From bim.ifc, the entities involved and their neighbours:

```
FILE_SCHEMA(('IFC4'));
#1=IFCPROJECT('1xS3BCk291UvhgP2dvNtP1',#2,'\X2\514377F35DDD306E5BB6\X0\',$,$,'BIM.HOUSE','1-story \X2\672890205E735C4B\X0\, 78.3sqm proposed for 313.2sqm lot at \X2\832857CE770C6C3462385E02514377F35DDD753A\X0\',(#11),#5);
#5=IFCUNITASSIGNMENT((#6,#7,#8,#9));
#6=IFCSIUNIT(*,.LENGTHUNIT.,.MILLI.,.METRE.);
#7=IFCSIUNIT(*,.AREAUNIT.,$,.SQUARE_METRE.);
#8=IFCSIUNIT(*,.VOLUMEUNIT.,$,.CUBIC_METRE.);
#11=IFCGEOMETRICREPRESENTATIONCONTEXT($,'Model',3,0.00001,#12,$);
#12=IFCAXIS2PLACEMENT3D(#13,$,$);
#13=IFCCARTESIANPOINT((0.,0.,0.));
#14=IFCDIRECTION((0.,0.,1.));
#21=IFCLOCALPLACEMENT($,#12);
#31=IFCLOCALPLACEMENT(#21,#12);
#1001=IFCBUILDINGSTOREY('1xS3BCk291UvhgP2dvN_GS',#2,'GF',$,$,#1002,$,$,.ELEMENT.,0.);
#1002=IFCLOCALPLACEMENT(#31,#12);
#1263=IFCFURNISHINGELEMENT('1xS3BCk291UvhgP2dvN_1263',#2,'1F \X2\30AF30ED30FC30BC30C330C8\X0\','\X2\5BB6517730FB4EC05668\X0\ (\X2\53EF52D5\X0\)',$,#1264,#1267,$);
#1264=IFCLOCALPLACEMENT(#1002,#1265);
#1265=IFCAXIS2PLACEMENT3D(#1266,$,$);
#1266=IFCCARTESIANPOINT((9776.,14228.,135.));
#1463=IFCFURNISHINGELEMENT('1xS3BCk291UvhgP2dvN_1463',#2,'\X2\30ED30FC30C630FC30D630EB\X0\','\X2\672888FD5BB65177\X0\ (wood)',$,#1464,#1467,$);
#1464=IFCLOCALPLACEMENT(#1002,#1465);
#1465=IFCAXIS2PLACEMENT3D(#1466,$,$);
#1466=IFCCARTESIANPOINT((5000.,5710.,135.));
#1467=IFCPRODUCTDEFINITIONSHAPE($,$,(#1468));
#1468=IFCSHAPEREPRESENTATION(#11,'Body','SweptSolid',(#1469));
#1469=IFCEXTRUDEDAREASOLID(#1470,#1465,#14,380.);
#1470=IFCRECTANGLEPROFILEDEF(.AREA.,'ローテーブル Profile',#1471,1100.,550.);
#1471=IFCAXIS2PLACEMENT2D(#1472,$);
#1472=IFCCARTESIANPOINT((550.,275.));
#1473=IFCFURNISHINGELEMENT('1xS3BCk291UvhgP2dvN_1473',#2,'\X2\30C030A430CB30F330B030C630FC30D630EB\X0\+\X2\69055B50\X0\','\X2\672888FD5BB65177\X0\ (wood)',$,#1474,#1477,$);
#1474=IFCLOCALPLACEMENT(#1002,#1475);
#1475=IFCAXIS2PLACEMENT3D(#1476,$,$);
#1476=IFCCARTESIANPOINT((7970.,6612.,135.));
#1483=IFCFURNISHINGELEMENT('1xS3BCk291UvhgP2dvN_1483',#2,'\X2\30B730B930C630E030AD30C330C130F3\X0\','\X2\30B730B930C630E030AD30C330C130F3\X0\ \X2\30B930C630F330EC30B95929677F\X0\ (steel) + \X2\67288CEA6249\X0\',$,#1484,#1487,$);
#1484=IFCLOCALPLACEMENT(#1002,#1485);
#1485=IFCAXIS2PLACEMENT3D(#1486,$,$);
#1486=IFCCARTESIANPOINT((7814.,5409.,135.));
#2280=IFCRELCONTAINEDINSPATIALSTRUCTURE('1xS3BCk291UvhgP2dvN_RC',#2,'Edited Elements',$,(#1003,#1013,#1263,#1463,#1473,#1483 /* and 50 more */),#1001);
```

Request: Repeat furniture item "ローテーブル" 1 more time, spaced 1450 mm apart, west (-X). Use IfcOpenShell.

```python
import numpy as np
import ifcopenshell
import ifcopenshell.api.geometry
import ifcopenshell.api.root
import ifcopenshell.util.element
import ifcopenshell.util.placement
import ifcopenshell.util.unit

model = ifcopenshell.open("bim.ifc")
unit_scale = ifcopenshell.util.unit.calculate_unit_scale(model)


def reuse_history(source, copy):
    """copy_class also copies each property set's owner history, people and application; keep the originals."""
    for rel in copy.IsDefinedBy:
        if rel.is_a("IfcRelDefinesByProperties") and (history := rel.RelatingPropertyDefinition.OwnerHistory):
            rel.RelatingPropertyDefinition.OwnerHistory = source.OwnerHistory
            ifcopenshell.util.element.remove_deep2(model, history)


source = model.by_guid("1xS3BCk291UvhgP2dvN_1463")
base = ifcopenshell.util.placement.get_local_placement(source.ObjectPlacement)
step = np.array([-1.0, 0.0, 0.0]) * 1.45 / unit_scale

for i in range(1, 2):
    copy = ifcopenshell.api.root.copy_class(model, product=source)
    copy.Representation = ifcopenshell.util.element.copy_deep(
        model, source.Representation, exclude=["IfcGeometricRepresentationContext", "IfcRepresentationMap"]
    )
    reuse_history(source, copy)
    matrix = base.copy()
    matrix[:3, 3] += i * step
    print("added at", matrix[:3, 3].round(3) + 0.0)
    ifcopenshell.api.geometry.edit_object_placement(model, product=copy, matrix=matrix, is_si=False)

model.write("bim_rev.ifc")
```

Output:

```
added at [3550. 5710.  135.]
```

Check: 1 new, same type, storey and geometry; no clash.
